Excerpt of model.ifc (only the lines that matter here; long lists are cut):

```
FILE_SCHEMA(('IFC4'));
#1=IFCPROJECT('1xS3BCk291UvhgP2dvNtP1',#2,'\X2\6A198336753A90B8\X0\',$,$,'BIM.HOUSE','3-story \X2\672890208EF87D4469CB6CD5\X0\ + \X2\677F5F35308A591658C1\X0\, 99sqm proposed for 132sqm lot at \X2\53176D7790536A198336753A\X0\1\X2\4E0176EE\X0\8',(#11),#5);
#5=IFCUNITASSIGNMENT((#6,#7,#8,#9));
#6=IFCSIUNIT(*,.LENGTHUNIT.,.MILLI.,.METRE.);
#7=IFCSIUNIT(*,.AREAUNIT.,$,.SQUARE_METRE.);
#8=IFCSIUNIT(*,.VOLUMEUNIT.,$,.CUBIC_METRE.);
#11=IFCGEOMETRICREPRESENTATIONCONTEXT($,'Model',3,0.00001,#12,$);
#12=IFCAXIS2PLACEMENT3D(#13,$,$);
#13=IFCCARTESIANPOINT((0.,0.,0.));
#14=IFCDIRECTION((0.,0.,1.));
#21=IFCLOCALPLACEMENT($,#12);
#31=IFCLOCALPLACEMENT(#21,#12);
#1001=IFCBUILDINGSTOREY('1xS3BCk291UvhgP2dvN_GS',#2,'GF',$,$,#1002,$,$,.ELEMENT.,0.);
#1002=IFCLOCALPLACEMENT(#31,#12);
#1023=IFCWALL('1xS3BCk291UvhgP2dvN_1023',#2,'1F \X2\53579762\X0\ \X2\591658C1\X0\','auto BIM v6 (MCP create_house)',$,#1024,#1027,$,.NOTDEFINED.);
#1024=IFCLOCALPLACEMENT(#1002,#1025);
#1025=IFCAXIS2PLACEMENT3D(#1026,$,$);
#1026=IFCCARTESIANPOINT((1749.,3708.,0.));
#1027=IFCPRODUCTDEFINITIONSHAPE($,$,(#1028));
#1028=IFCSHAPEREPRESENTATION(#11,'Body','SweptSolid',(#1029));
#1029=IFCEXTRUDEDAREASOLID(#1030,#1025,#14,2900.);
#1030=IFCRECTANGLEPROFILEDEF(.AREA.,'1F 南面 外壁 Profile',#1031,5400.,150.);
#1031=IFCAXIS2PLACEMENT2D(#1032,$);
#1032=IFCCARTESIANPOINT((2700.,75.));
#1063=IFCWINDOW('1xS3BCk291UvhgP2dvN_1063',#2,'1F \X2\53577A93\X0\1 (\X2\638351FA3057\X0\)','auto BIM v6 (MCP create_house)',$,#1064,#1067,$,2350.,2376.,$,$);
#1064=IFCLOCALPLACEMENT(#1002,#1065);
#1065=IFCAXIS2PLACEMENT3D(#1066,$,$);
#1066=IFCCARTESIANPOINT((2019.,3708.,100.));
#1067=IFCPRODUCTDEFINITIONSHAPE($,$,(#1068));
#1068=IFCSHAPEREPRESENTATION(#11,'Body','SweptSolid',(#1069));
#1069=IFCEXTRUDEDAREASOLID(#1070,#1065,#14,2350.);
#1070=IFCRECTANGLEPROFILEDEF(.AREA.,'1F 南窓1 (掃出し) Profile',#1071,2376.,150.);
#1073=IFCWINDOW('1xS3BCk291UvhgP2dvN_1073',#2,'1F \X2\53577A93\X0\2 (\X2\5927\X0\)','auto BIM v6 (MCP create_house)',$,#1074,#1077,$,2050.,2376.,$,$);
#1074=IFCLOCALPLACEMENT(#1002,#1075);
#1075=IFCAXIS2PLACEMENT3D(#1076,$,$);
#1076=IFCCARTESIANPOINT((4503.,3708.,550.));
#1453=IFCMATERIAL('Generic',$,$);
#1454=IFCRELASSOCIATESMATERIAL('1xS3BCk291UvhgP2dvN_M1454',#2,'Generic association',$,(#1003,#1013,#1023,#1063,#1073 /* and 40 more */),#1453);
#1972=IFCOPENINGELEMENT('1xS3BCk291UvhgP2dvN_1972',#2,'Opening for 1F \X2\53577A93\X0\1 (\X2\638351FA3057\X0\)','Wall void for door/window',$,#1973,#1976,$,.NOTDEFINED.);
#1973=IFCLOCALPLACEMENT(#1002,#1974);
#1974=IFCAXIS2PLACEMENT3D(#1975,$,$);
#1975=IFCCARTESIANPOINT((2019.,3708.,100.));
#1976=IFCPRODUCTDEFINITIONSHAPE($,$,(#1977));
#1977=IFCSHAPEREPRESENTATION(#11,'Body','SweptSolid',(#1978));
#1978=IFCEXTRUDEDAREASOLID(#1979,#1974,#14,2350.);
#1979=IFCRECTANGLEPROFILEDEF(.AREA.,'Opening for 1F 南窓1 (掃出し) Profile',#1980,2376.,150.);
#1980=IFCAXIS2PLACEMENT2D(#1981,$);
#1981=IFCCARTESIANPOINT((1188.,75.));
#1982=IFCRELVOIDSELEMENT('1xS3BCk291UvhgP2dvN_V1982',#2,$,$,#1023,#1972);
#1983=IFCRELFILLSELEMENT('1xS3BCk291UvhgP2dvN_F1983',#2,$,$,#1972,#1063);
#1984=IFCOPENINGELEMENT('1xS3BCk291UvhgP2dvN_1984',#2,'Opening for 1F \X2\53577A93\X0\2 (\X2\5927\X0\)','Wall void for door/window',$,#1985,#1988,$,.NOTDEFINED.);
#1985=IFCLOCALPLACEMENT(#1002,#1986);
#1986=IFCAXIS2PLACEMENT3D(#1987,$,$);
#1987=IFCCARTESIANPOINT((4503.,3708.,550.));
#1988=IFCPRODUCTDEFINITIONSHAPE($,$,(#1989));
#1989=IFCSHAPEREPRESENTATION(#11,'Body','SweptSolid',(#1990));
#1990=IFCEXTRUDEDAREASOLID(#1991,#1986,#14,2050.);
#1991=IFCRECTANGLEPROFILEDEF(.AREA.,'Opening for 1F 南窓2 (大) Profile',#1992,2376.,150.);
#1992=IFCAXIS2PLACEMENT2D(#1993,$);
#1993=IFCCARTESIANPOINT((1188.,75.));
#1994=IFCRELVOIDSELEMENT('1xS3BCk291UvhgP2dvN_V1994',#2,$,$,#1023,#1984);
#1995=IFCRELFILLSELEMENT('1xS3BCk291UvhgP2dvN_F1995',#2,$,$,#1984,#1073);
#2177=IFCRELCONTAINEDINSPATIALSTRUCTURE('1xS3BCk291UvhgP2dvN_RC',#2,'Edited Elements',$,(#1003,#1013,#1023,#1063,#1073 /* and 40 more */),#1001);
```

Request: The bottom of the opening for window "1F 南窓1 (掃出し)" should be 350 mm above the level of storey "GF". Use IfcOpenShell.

```python
import numpy as np
import ifcopenshell
import ifcopenshell.api.geometry
import ifcopenshell.geom
import ifcopenshell.util.element
import ifcopenshell.util.placement
import ifcopenshell.util.shape
import ifcopenshell.util.unit

model = ifcopenshell.open("model.ifc")
unit_scale = ifcopenshell.util.unit.calculate_unit_scale(model)

window = model.by_id(1063)
opening = window.FillsVoids[0].RelatingOpeningElement
storey = ifcopenshell.util.element.get_container(window, ifc_class="IfcBuildingStorey")
level = ifcopenshell.util.placement.get_local_placement(storey.ObjectPlacement)[2, 3]

# The opening's origin need not be at the sill, so measure its lowest point.
shape = ifcopenshell.geom.create_shape(ifcopenshell.geom.settings(), opening)
bottom = ifcopenshell.util.shape.get_shape_bottom_elevation(shape, shape.geometry) / unit_scale
dz = level + 0.35 / unit_scale - bottom

shift = np.array([0.0, 0.0, dz])
# The window is not placed relative to its opening, so move both.
for product in (opening, window):
    matrix = ifcopenshell.util.placement.get_local_placement(product.ObjectPlacement)
    matrix[:3, 3] += shift
    ifcopenshell.api.geometry.edit_object_placement(model, product=product, matrix=matrix, is_si=False)

print(f"moved by {dz * unit_scale:+.3f} m")

model.write("model_updated.ifc")
```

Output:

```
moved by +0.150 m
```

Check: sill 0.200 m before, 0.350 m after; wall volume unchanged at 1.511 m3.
